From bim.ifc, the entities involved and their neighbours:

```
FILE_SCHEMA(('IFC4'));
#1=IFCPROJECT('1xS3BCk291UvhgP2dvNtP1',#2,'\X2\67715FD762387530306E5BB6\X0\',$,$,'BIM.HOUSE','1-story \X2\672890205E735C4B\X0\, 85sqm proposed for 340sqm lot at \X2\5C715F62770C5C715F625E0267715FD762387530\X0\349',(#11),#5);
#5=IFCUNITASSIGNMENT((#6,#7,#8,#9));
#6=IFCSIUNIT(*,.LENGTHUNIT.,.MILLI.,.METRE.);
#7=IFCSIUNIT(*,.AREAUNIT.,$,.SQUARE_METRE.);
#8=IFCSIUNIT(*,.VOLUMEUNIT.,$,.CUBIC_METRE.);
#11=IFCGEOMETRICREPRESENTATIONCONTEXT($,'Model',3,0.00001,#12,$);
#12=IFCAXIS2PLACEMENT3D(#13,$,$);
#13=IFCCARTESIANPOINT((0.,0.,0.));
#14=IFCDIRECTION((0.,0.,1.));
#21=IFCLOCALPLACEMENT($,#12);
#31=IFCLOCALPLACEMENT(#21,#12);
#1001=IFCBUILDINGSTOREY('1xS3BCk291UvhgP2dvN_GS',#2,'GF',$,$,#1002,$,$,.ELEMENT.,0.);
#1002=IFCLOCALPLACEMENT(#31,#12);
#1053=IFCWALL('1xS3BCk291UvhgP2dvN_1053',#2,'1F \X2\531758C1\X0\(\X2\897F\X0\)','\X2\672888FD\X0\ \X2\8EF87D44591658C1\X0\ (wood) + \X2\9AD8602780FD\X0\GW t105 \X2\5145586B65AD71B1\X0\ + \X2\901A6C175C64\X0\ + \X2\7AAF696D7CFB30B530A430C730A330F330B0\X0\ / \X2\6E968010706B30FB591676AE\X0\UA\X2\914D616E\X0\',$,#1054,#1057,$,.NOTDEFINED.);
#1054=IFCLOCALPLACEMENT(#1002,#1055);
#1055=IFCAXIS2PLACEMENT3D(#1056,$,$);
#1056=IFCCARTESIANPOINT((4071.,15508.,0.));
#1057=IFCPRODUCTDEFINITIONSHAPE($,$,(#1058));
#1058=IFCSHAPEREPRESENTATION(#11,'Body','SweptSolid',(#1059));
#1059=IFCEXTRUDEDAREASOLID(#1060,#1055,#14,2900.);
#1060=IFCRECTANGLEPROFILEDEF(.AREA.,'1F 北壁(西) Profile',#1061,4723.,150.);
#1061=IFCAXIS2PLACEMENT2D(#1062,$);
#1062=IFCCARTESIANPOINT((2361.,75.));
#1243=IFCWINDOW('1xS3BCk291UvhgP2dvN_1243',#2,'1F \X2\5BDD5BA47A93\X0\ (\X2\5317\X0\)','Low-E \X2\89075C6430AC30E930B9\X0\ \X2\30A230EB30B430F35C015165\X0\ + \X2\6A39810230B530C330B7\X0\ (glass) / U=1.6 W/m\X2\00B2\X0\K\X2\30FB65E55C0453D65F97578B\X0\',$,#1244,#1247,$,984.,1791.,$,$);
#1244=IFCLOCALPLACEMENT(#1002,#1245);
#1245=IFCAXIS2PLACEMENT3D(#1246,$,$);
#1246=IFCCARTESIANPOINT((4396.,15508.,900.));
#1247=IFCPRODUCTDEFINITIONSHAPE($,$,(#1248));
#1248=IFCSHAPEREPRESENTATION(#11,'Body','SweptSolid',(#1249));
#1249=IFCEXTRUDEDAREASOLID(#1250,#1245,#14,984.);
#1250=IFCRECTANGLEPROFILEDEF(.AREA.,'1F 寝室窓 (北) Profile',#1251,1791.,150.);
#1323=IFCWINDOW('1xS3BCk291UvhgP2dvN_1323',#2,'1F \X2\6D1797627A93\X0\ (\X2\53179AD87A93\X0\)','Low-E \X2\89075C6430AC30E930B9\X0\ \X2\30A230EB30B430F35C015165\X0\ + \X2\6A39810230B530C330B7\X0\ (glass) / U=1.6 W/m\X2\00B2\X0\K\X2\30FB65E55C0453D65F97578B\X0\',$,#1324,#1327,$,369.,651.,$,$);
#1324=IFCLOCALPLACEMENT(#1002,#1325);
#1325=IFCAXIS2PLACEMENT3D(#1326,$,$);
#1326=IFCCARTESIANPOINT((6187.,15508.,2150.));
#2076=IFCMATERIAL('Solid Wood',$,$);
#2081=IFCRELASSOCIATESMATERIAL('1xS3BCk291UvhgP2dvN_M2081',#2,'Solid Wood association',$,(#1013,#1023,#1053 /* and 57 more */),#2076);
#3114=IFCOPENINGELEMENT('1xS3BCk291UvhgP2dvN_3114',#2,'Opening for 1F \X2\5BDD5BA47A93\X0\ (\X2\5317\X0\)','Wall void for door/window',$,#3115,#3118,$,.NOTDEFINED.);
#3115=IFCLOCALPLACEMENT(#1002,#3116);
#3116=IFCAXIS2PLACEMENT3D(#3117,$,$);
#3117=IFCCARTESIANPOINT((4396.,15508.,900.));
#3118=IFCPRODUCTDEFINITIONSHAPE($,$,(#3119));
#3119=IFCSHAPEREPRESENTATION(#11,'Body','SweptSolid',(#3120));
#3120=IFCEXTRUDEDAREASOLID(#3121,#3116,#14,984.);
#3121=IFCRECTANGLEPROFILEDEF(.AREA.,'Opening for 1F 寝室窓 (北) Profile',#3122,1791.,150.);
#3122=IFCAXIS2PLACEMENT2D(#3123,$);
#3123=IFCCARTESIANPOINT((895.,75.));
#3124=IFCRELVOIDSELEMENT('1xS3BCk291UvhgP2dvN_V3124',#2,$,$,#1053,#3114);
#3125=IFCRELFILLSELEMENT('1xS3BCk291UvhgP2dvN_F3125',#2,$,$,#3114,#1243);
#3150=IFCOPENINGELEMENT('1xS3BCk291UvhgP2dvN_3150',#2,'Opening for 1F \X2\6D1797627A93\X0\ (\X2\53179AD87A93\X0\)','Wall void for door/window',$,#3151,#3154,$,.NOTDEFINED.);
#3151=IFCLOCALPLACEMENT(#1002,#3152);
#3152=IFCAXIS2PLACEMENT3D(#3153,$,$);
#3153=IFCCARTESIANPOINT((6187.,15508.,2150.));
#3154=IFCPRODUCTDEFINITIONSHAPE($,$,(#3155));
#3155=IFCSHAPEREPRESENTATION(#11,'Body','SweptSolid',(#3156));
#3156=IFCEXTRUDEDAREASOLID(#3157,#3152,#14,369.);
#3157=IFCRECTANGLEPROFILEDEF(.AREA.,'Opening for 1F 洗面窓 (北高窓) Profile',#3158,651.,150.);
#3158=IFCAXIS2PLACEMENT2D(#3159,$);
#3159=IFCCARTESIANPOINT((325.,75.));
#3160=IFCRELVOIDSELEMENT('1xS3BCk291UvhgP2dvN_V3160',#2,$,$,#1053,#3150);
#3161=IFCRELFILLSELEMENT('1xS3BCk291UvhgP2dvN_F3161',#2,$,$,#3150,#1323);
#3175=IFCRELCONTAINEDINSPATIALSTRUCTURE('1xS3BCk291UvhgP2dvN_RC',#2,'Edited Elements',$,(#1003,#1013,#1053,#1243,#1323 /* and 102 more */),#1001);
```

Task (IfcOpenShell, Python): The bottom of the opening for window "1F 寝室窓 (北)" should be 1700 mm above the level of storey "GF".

```python
import numpy as np
import ifcopenshell
import ifcopenshell.api.geometry
import ifcopenshell.geom
import ifcopenshell.util.element
import ifcopenshell.util.placement
import ifcopenshell.util.shape
import ifcopenshell.util.unit

model = ifcopenshell.open("bim.ifc")
unit_scale = ifcopenshell.util.unit.calculate_unit_scale(model)

window = model.by_guid("1xS3BCk291UvhgP2dvN_1243")
opening = window.FillsVoids[0].RelatingOpeningElement
storey = ifcopenshell.util.element.get_container(window, ifc_class="IfcBuildingStorey")
level = ifcopenshell.util.placement.get_local_placement(storey.ObjectPlacement)[2, 3]

# The opening's origin need not be at the sill, so measure its lowest point.
shape = ifcopenshell.geom.create_shape(ifcopenshell.geom.settings(), opening)
bottom = ifcopenshell.util.shape.get_shape_bottom_elevation(shape, shape.geometry) / unit_scale
dz = level + 1.7 / unit_scale - bottom

shift = np.array([0.0, 0.0, dz])
# The window is not placed relative to its opening, so move both.
for product in (opening, window):
    matrix = ifcopenshell.util.placement.get_local_placement(product.ObjectPlacement)
    matrix[:3, 3] += shift
    ifcopenshell.api.geometry.edit_object_placement(model, product=product, matrix=matrix, is_si=False)

print(f"moved by {dz * unit_scale:+.3f} m")

model.write("bim_edited.ifc")
```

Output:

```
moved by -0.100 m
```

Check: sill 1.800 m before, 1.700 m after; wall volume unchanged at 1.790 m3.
